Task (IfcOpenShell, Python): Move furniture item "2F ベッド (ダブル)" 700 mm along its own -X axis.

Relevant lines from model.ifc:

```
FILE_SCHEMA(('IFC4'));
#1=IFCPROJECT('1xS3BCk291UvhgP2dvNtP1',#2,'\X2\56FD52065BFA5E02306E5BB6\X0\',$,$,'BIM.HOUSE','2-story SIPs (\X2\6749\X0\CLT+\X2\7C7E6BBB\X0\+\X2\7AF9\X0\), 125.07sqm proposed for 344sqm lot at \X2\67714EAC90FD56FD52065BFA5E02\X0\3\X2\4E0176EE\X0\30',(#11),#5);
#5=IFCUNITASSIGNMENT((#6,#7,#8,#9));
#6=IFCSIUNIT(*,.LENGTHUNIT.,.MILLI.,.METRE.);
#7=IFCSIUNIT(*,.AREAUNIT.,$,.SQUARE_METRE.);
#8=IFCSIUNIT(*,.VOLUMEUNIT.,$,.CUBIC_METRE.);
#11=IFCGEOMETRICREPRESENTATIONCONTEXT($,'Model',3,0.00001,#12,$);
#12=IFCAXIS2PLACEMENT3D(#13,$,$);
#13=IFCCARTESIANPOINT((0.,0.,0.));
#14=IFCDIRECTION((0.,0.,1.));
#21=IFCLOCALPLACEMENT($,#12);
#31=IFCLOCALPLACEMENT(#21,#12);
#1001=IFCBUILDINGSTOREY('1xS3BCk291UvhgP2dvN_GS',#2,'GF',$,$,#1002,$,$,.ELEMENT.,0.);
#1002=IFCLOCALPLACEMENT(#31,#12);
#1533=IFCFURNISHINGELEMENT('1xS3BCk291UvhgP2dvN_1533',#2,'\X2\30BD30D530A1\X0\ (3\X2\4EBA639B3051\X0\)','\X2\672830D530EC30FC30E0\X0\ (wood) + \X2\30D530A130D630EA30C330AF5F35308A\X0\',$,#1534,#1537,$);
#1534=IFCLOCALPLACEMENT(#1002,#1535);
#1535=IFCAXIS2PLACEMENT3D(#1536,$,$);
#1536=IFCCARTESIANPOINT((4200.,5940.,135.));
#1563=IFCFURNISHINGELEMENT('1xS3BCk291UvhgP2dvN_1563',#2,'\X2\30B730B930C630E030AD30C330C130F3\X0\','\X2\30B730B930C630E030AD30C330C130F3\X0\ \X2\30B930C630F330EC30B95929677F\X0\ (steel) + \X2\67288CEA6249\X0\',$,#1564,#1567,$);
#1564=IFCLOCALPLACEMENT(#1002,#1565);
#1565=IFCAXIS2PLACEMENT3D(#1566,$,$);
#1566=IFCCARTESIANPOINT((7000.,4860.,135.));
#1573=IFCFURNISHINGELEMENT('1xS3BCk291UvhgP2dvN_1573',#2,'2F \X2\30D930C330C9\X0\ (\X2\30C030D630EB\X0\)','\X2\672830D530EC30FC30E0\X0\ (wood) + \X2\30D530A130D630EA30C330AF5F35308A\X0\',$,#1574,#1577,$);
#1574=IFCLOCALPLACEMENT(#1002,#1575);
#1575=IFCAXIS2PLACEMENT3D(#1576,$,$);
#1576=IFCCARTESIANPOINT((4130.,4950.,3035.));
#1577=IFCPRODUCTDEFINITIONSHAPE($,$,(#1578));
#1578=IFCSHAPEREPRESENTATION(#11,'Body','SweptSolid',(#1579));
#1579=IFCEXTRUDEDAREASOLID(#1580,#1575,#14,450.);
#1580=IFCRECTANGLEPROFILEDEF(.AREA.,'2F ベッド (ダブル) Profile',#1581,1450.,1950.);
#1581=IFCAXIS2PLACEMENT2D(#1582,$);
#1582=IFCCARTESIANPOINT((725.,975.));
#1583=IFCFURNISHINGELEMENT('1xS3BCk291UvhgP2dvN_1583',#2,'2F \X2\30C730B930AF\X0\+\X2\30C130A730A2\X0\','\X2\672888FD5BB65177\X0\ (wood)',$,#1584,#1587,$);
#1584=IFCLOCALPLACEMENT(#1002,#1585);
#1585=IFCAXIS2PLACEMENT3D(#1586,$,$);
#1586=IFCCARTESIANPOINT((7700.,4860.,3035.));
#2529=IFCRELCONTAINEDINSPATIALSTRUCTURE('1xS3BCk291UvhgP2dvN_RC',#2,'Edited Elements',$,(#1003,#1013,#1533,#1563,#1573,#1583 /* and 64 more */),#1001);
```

```python
import ifcopenshell
import ifcopenshell.api.geometry
import ifcopenshell.util.placement
import ifcopenshell.util.unit

model = ifcopenshell.open("model.ifc")
unit_scale = ifcopenshell.util.unit.calculate_unit_scale(model)

item = model.by_id(1573)
matrix = ifcopenshell.util.placement.get_local_placement(item.ObjectPlacement)
matrix[:3, 3] -= matrix[:3, 0] * 0.7 / unit_scale
ifcopenshell.api.geometry.edit_object_placement(model, product=item, matrix=matrix, is_si=False)

print(ifcopenshell.util.placement.get_local_placement(item.ObjectPlacement).round(3) + 0.0)

model.write("model_edited.ifc")
```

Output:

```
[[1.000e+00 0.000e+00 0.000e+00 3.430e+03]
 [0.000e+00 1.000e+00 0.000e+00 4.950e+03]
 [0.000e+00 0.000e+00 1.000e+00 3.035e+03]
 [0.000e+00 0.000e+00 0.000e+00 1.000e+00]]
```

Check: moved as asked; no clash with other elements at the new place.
